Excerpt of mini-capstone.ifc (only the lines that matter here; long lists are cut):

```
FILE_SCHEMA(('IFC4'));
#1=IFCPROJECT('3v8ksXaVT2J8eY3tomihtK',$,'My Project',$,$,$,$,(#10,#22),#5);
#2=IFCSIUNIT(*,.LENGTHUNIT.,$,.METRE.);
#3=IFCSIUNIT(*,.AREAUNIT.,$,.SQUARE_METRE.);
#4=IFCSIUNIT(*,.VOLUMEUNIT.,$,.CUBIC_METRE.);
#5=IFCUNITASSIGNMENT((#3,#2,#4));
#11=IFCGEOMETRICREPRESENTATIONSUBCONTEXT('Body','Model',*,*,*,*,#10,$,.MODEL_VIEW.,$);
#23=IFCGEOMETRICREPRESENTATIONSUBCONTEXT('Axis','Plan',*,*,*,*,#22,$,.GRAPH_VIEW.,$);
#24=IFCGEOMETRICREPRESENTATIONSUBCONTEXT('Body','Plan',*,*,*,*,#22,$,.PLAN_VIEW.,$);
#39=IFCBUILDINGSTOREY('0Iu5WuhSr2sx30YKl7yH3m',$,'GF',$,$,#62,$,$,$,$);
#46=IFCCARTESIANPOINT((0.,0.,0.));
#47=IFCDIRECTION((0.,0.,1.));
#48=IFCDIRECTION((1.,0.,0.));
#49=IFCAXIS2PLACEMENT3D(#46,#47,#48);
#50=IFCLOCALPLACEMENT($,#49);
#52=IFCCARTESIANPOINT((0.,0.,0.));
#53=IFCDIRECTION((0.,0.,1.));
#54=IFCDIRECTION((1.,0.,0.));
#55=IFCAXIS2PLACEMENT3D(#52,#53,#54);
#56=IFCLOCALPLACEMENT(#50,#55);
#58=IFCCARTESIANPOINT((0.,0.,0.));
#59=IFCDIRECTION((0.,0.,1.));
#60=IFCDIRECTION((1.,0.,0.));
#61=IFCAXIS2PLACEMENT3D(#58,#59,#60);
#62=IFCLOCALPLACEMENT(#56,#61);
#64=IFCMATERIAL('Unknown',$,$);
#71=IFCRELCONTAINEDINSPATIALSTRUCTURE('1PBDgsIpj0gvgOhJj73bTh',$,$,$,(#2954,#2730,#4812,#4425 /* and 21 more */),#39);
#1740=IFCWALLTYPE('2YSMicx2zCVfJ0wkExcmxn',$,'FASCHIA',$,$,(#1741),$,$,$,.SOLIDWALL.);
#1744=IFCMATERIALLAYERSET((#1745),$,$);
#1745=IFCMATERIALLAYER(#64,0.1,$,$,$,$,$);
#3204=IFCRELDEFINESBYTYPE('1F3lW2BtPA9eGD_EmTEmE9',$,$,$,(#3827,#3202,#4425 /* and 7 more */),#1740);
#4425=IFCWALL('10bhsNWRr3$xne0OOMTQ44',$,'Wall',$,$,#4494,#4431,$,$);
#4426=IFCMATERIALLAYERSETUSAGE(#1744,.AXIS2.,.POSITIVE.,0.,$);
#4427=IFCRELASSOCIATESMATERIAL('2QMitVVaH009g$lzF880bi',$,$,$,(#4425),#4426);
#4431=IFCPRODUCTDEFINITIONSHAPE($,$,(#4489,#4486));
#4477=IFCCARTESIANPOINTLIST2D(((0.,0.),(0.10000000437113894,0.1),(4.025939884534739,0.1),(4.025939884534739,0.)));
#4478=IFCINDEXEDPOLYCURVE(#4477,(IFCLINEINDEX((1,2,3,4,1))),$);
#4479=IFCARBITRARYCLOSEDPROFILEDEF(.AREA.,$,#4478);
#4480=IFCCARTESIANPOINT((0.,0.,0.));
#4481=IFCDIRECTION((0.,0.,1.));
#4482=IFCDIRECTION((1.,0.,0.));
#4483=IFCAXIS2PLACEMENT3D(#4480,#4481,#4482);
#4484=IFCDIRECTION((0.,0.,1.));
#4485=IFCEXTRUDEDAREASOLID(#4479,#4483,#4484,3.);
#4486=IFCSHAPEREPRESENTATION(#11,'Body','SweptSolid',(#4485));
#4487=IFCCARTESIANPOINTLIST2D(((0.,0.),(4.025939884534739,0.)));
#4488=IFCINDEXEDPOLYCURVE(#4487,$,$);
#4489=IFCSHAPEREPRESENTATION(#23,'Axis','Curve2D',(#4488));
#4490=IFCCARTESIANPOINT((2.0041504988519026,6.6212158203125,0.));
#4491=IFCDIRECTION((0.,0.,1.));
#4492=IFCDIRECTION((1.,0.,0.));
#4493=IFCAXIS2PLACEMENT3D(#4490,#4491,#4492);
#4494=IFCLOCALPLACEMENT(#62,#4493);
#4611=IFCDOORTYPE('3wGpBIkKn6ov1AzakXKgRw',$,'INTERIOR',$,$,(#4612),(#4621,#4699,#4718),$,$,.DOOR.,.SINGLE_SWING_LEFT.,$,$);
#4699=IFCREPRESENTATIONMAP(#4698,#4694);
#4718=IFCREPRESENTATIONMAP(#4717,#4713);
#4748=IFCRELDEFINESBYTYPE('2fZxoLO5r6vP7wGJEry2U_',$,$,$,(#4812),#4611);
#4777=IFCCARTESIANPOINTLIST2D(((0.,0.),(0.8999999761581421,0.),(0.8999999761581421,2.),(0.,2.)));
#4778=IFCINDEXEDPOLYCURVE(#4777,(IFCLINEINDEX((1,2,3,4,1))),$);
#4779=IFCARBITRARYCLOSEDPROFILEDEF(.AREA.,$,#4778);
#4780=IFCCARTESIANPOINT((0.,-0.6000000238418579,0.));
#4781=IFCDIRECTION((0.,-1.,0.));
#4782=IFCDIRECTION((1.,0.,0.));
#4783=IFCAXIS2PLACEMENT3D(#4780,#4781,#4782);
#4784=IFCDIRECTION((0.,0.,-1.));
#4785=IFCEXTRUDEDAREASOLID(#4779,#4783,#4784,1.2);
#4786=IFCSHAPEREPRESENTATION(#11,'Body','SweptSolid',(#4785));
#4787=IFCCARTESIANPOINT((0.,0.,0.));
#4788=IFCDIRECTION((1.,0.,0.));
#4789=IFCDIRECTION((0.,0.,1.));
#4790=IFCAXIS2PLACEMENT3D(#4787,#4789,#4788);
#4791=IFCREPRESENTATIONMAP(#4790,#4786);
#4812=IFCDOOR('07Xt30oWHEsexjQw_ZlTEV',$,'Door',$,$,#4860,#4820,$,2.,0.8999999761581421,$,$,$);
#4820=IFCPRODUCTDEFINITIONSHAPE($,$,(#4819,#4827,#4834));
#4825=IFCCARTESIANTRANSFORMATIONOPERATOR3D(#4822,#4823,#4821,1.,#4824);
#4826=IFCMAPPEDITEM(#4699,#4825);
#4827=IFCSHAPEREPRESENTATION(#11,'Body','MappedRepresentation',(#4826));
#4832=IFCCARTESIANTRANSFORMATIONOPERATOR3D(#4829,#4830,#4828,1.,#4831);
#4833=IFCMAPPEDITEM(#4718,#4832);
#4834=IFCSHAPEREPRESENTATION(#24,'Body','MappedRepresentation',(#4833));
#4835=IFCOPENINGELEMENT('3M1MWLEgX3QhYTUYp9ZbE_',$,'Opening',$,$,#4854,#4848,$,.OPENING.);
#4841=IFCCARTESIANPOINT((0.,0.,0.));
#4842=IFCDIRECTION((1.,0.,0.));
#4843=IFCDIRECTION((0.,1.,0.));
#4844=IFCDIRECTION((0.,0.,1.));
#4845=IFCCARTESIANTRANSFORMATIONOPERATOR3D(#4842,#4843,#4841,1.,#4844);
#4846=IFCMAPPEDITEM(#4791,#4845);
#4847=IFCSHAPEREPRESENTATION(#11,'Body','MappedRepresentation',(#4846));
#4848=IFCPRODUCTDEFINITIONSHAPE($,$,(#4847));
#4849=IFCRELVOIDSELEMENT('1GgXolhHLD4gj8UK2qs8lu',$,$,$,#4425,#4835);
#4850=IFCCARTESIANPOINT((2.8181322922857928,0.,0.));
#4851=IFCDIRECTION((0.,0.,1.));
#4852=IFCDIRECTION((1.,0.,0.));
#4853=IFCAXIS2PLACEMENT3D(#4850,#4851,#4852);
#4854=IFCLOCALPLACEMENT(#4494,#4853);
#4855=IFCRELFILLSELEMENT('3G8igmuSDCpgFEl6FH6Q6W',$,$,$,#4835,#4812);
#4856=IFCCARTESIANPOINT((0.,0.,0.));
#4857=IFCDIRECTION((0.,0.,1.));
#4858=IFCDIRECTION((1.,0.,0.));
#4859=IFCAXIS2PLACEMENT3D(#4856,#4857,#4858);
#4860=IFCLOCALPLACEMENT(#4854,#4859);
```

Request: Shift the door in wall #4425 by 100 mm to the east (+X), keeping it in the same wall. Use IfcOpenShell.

```python
import ifcopenshell
import ifcopenshell.api.geometry
import ifcopenshell.util.placement

model = ifcopenshell.open("mini-capstone.ifc")

door = model.by_guid("07Xt30oWHEsexjQw_ZlTEV")
opening = door.FillsVoids[0].RelatingOpeningElement
wall = opening.VoidsElements[0].RelatingBuildingElement

wall_matrix = ifcopenshell.util.placement.get_local_placement(wall.ObjectPlacement)
shift = wall_matrix[:3, 0] * 0.1
before = ifcopenshell.util.placement.get_local_placement(door.ObjectPlacement)[:3, 3].copy()

# The door is placed relative to its opening, so it follows when the opening moves.
matrix = ifcopenshell.util.placement.get_local_placement(opening.ObjectPlacement)
matrix[:3, 3] += shift
ifcopenshell.api.geometry.edit_object_placement(
    model, product=opening, matrix=matrix, is_si=False, should_transform_children=True
)

after = ifcopenshell.util.placement.get_local_placement(door.ObjectPlacement)[:3, 3]
print("door moved by", (after - before).round(3) + 0.0)

model.write("mini-capstone_edited.ifc")
```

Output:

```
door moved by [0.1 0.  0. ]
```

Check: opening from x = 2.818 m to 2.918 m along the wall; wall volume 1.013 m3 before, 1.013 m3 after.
